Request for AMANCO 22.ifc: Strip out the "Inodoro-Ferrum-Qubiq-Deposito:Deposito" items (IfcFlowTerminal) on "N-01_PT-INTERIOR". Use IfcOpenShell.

First a look at what the model holds.

```python
import ifcopenshell
import ifcopenshell.util.element

model = ifcopenshell.open("AMANCO 22.ifc")
print(model.schema)
storey = next(s for s in model.by_type("IfcBuildingStorey") if s.Name == "N-01_PT-INTERIOR")
terminals = [e for e in ifcopenshell.util.element.get_decomposition(storey) if e.is_a("IfcFlowTerminal")]
seen = {}
for e in terminals:
    element_type = ifcopenshell.util.element.get_type(e)
    name = element_type.Name if element_type not in (None, e) else None
    seen[name] = seen.get(name, 0) + 1
for name, count in sorted(seen.items(), key=str):
    print(count, "x", name)
```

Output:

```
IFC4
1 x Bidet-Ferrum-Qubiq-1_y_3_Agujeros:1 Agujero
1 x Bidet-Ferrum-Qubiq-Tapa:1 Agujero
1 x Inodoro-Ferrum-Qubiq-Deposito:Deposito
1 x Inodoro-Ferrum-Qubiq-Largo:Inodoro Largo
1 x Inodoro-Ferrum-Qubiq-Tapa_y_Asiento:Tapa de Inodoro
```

```python
import ifcopenshell
import ifcopenshell.api.root
import ifcopenshell.util.element

model = ifcopenshell.open("AMANCO 22.ifc")

storey = next(s for s in model.by_type("IfcBuildingStorey") if s.Name == "N-01_PT-INTERIOR")
terminals = [e for e in ifcopenshell.util.element.get_decomposition(storey) if e.is_a("IfcFlowTerminal")]
targets = [e for e in terminals if (t := ifcopenshell.util.element.get_type(e)) not in (None, e) and t.Name == "Inodoro-Ferrum-Qubiq-Deposito:Deposito"]

for e in targets:
    ifcopenshell.api.root.remove_product(model, product=e)
print(len(targets), "removed")

model.write("AMANCO 22-out.ifc")
```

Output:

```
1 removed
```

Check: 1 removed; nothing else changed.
